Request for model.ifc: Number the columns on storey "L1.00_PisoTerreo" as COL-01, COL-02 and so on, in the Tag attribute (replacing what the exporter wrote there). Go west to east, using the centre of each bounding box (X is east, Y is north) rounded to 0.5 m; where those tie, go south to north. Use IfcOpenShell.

First a look at what the model holds.

```python
import ifcopenshell
import ifcopenshell.util.element
import ifcopenshell.util.placement

model = ifcopenshell.open("model.ifc")
print(model.schema)
storey = next(s for s in model.by_type("IfcBuildingStorey") if s.Name == "L1.00_PisoTerreo")
columns = [e for e in ifcopenshell.util.element.get_decomposition(storey) if e.is_a("IfcColumn")]
for e in sorted(columns, key=lambda e: e.id()):
    origin = ifcopenshell.util.placement.get_local_placement(e.ObjectPlacement)[:3, 3]
    print(e.id(), e.Tag, e.Name, origin.round(2) + 0.0, sep=" | ")
```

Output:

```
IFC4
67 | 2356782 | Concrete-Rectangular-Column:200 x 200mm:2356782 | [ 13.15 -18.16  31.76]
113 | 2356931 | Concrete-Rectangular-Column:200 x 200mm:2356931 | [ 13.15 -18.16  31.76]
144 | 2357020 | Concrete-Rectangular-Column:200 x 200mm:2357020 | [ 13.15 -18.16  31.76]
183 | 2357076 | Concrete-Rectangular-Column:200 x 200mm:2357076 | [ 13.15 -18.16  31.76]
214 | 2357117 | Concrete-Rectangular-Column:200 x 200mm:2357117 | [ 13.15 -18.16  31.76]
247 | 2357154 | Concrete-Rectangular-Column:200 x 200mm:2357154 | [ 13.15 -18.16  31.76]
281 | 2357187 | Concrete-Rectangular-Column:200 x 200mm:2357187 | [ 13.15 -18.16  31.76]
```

```python
import ifcopenshell
import ifcopenshell.geom
import ifcopenshell.util.element
import ifcopenshell.util.shape

model = ifcopenshell.open("model.ifc")
settings = ifcopenshell.geom.settings()
settings.set("use-world-coords", True)


def centre(element):
    shape = ifcopenshell.geom.create_shape(settings, element)
    return ifcopenshell.util.shape.get_bbox_centroid(shape.geometry)


storey = next(s for s in model.by_type("IfcBuildingStorey") if s.Name == "L1.00_PisoTerreo")
columns = [e for e in ifcopenshell.util.element.get_decomposition(storey) if e.is_a("IfcColumn")]

# Insertion points can sit at a corner or the storey origin, so sort by the geometry (in metres).
centres = {e: centre(e) for e in columns}
columns.sort(key=lambda e: (round(centres[e][0] / 0.5), centres[e][1]))

for i, e in enumerate(columns, start=1):
    number = f"COL-{i:02d}"
    e.Tag = number
    print(e.id(), number)

model.write("model_v2.ifc")
```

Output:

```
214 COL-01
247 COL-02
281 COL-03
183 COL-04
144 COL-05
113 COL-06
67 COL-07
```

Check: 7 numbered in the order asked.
